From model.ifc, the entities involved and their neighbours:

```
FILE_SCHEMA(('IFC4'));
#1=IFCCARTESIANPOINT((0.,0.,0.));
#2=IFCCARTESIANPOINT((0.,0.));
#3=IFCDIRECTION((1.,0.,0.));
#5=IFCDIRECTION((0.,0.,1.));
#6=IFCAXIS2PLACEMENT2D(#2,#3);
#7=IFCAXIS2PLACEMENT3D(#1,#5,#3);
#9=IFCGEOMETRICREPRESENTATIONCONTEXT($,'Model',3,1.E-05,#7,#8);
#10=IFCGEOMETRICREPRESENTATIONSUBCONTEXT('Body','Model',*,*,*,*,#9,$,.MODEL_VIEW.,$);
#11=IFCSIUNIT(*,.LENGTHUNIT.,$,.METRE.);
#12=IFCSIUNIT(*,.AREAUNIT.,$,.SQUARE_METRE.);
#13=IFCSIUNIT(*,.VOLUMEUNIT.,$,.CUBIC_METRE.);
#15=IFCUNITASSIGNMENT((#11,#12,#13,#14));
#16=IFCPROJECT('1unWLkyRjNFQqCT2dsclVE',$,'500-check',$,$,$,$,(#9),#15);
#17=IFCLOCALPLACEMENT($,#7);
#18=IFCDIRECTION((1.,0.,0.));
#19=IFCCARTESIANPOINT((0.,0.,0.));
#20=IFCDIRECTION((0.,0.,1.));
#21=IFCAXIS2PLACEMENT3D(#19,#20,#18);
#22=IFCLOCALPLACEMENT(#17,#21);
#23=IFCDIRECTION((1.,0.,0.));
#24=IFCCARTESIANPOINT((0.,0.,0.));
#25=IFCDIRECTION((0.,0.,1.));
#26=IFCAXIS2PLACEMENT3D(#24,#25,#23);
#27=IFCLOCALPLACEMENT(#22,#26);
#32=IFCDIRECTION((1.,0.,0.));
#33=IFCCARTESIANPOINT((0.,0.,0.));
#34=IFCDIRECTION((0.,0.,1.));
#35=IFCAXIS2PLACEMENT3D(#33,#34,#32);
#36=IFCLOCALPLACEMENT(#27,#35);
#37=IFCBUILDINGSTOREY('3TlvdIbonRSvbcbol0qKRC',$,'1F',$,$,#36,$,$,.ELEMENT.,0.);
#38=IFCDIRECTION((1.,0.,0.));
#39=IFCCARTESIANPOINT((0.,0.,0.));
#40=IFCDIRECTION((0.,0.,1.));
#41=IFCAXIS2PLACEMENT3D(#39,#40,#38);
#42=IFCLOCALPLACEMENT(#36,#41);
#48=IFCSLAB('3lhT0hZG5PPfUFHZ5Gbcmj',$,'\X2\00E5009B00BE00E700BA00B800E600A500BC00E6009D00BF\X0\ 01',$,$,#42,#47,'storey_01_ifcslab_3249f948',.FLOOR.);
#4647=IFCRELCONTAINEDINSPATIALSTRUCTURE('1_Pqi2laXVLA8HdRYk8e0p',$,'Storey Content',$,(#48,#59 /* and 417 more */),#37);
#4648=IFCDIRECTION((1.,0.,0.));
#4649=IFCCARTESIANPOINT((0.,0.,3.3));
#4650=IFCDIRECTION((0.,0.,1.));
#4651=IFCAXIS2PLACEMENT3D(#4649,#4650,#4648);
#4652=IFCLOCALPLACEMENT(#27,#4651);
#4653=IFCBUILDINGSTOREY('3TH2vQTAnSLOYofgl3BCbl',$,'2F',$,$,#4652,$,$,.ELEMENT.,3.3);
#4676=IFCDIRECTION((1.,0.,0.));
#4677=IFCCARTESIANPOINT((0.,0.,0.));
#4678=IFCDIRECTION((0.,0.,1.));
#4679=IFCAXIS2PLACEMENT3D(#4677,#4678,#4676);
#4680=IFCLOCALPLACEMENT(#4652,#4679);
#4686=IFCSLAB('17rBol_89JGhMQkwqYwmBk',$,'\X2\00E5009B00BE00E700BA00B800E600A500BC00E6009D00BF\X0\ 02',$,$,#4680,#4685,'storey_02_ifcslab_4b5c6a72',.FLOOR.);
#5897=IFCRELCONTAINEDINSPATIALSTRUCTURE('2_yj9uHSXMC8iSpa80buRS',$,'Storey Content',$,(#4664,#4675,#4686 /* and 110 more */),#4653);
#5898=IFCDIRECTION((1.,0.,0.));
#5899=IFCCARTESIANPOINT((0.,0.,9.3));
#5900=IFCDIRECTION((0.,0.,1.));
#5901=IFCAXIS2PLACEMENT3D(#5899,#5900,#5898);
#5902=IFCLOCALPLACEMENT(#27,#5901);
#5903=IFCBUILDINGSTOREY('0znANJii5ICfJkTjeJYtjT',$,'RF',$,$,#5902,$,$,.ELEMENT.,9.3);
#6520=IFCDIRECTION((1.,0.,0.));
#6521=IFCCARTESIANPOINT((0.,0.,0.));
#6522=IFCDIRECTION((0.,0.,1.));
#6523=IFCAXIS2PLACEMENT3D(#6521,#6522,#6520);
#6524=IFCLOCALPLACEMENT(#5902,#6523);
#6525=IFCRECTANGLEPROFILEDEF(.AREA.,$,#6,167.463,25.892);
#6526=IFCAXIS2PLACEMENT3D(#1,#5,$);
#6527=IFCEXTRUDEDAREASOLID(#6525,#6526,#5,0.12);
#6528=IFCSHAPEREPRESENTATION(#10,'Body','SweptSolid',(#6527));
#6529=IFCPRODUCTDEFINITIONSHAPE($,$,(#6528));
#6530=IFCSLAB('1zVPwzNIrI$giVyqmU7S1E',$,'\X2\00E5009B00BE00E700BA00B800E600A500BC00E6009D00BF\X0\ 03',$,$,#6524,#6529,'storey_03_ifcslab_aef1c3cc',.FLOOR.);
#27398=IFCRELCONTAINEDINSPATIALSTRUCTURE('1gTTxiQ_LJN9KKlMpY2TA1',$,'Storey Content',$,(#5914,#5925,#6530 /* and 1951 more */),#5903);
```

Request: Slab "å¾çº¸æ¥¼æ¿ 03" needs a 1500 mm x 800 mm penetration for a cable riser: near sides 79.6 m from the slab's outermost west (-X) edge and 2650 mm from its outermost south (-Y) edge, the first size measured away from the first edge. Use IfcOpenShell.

```python
import numpy as np
import ifcopenshell
import ifcopenshell.api.feature
import ifcopenshell.api.geometry
import ifcopenshell.api.root
import ifcopenshell.geom
import ifcopenshell.util.placement
import ifcopenshell.util.representation
import ifcopenshell.util.shape
import ifcopenshell.util.unit

model = ifcopenshell.open("model.ifc")
unit_scale = ifcopenshell.util.unit.calculate_unit_scale(model)
settings = ifcopenshell.geom.settings()


def volume(element):
    """Net volume in cubic metres, openings subtracted."""
    shape = ifcopenshell.geom.create_shape(settings, element)
    return ifcopenshell.util.shape.get_volume(shape.geometry)


slab = model.by_guid("1zVPwzNIrI$giVyqmU7S1E")
before = volume(slab)

# Extent in the slab's own axes, in metres. The edges named are its -X and -Y sides.
slab_shape = ifcopenshell.geom.create_shape(settings, slab)
vertices = ifcopenshell.util.shape.get_vertices(slab_shape.geometry)
x_min, y_min, bottom = vertices.min(axis=0)
top = vertices[:, 2].max()

opening = ifcopenshell.api.root.create_entity(model, ifc_class="IfcOpeningElement", name="Cable riser opening", predefined_type="OPENING")
context = ifcopenshell.util.representation.get_context(model, "Model", "Body", "MODEL_VIEW")
width, depth = 1.5, 0.8
outline = [(0.0, 0.0), (width, 0.0), (width, depth), (0.0, depth), (0.0, 0.0)]
# Overshoot both faces by 50 mm so the cut is clean.
shape = ifcopenshell.api.geometry.add_slab_representation(
    model, context=context, depth=top - bottom + 0.1, polyline=outline
)
ifcopenshell.api.geometry.assign_representation(model, product=opening, representation=shape)

matrix = ifcopenshell.util.placement.get_local_placement(slab.ObjectPlacement)
matrix[:, 3] = matrix @ np.append(np.array([x_min + 79.6, y_min + 2.65, bottom - 0.05]) / unit_scale, 1.0)
ifcopenshell.api.geometry.edit_object_placement(model, product=opening, matrix=matrix, is_si=False)
ifcopenshell.api.feature.add_feature(model, feature=opening, element=slab)

after = volume(slab)

print(f"slab volume {before:.3f} -> {after:.3f} m3")

model.write("model-out.ifc")
```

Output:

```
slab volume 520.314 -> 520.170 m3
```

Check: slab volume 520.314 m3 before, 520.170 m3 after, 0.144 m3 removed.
